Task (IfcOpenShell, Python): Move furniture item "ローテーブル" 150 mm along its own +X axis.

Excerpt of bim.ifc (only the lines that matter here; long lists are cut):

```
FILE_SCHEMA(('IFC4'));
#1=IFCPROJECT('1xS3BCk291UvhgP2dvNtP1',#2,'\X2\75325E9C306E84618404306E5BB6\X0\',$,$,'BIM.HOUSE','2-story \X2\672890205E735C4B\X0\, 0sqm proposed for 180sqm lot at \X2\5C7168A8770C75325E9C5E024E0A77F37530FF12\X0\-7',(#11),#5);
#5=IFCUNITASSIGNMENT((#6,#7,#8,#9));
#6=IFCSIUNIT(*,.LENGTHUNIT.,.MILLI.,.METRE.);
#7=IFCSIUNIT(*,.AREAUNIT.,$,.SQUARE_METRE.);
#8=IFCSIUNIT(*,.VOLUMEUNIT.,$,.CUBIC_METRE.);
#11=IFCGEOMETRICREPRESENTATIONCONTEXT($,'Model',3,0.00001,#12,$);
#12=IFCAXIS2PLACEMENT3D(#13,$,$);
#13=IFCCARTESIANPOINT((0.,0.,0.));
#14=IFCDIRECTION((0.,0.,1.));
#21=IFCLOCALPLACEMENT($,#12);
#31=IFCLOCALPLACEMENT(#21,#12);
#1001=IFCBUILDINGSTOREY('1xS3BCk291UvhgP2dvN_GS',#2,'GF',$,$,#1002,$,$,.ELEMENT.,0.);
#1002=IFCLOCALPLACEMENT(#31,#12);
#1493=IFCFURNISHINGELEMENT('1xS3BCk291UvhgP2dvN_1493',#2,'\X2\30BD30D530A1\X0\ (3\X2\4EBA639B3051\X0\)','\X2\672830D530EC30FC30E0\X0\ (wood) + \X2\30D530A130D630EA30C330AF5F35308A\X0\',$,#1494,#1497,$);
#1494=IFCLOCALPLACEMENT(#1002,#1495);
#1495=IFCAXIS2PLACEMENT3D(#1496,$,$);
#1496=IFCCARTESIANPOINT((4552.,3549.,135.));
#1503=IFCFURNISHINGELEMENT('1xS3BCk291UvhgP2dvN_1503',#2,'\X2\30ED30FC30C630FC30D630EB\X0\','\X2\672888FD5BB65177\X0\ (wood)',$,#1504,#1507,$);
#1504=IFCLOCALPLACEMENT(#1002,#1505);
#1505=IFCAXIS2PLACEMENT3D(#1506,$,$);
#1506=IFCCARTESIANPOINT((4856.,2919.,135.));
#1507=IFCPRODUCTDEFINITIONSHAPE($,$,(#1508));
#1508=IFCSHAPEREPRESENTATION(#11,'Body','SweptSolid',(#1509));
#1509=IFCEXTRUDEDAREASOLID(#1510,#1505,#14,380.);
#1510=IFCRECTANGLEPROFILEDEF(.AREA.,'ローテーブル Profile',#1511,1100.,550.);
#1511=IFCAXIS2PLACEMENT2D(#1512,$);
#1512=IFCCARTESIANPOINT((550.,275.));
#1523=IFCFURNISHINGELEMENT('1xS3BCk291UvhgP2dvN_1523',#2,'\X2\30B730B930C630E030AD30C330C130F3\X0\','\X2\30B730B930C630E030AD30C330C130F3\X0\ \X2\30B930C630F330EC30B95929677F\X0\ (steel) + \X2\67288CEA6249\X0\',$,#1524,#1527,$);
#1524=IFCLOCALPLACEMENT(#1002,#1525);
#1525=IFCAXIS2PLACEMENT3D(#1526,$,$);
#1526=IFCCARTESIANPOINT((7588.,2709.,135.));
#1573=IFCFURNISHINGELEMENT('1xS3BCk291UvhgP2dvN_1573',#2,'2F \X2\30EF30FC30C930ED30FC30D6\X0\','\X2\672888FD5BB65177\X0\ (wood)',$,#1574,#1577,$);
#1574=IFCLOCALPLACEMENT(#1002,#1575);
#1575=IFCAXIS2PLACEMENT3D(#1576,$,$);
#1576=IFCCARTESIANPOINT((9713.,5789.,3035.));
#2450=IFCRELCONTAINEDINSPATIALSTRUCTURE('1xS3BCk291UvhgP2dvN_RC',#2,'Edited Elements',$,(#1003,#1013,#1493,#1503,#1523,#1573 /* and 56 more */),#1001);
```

```python
import ifcopenshell
import ifcopenshell.api.geometry
import ifcopenshell.util.placement

model = ifcopenshell.open("bim.ifc")

item = model.by_guid("1xS3BCk291UvhgP2dvN_1503")
matrix = ifcopenshell.util.placement.get_local_placement(item.ObjectPlacement)
matrix[:3, 3] += matrix[:3, 0] * 150.0
ifcopenshell.api.geometry.edit_object_placement(model, product=item, matrix=matrix, is_si=False)

print(ifcopenshell.util.placement.get_local_placement(item.ObjectPlacement).round(3) + 0.0)

model.write("bim_rev.ifc")
```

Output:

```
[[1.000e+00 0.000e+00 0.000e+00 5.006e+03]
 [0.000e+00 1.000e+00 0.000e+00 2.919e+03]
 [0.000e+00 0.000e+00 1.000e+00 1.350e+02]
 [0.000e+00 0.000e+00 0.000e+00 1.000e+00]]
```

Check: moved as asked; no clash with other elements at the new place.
